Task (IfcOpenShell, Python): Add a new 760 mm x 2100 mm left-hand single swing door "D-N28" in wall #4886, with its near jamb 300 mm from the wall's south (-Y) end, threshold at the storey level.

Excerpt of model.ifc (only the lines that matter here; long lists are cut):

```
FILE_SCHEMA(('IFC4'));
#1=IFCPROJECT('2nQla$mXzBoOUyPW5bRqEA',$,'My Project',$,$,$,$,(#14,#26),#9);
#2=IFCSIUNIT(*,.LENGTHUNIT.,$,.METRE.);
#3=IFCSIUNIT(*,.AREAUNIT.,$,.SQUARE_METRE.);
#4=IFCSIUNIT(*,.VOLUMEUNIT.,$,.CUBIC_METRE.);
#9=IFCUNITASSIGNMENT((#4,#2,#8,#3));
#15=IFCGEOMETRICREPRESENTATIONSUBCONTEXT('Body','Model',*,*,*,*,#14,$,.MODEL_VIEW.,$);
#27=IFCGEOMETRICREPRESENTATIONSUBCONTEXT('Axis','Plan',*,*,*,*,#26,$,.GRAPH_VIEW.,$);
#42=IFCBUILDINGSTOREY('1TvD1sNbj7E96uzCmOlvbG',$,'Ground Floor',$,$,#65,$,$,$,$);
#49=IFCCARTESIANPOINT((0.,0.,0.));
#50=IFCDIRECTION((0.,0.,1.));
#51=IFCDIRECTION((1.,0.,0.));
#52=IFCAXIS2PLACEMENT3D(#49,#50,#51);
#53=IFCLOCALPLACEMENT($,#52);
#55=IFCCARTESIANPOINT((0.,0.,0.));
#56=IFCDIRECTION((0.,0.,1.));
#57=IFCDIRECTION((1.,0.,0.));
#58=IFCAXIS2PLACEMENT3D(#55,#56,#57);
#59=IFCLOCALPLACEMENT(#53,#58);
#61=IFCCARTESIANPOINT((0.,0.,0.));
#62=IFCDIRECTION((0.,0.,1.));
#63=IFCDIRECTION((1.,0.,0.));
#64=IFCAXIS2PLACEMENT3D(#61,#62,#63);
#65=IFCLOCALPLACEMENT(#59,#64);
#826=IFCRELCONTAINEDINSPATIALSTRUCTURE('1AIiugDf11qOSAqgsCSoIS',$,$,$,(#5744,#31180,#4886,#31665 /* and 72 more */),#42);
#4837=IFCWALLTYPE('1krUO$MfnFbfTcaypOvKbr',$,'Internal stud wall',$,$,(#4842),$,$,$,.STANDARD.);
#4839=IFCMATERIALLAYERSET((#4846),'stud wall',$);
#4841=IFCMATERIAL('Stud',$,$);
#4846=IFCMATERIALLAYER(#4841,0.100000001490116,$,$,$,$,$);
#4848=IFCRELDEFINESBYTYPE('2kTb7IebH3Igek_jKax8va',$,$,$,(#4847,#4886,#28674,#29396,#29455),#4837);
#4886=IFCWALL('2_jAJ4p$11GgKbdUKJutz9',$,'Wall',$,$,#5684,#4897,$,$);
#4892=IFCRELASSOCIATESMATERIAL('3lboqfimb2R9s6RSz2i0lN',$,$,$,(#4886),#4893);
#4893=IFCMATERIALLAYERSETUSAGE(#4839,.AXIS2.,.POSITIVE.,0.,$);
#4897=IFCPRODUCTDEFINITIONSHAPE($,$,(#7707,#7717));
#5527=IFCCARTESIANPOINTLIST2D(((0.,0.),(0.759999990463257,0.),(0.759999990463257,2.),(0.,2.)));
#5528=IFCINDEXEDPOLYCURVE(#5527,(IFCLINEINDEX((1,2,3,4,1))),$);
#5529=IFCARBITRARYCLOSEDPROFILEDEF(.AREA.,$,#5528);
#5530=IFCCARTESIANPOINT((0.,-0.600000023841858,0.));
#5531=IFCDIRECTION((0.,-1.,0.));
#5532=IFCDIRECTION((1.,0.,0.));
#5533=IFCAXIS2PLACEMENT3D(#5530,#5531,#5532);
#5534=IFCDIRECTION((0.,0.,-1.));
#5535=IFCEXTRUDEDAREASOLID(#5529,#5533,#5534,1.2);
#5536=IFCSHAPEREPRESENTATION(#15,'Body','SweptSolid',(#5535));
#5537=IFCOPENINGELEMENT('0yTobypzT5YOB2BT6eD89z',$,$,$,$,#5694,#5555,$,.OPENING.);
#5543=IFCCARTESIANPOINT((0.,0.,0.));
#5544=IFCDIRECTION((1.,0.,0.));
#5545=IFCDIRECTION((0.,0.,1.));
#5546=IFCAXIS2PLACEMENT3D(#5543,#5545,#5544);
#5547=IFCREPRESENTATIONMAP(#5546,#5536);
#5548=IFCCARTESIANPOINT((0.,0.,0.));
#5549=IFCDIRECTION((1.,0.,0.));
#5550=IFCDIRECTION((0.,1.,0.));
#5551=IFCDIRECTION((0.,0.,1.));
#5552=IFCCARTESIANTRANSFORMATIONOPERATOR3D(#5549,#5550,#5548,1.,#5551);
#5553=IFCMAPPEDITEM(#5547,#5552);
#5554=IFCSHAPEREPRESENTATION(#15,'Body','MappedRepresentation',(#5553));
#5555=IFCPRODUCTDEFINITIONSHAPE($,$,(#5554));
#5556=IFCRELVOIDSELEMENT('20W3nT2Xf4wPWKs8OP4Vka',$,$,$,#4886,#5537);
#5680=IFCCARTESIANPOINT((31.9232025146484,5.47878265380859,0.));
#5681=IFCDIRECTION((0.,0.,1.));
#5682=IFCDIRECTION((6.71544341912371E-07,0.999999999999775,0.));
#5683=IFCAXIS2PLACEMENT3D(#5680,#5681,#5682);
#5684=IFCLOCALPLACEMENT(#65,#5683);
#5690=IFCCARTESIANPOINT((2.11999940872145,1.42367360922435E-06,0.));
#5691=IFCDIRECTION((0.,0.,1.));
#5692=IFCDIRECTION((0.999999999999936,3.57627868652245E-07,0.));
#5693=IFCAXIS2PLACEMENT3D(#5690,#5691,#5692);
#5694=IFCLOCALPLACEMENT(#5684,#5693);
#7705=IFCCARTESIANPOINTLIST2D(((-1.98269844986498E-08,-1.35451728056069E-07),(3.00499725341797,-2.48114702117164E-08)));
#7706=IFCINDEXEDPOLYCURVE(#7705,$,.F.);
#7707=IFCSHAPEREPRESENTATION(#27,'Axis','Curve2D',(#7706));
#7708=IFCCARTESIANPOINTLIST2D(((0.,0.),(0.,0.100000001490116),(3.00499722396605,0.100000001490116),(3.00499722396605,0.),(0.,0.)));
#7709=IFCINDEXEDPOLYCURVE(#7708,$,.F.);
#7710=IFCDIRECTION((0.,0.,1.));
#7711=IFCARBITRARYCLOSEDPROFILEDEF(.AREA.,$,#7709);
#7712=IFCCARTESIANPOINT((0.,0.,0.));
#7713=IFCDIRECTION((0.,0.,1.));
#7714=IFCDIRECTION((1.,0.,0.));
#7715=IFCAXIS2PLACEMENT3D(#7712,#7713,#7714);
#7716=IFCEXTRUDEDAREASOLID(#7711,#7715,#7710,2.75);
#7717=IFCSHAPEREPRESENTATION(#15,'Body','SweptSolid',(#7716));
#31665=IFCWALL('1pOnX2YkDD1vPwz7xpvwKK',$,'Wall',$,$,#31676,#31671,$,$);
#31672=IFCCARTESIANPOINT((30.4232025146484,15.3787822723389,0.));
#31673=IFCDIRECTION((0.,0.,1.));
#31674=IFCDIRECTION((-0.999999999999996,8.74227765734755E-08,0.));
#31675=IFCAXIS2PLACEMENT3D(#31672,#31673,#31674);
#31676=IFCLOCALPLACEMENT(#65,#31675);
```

```python
import numpy as np
import ifcopenshell
import ifcopenshell.api.feature
import ifcopenshell.api.geometry
import ifcopenshell.api.root
import ifcopenshell.api.spatial
import ifcopenshell.geom
import ifcopenshell.util.element
import ifcopenshell.util.placement
import ifcopenshell.util.representation
import ifcopenshell.util.shape
import ifcopenshell.util.unit

model = ifcopenshell.open("model.ifc")
unit_scale = ifcopenshell.util.unit.calculate_unit_scale(model)
settings = ifcopenshell.geom.settings()


def volume(element):
    """Net volume in cubic metres, openings subtracted."""
    shape = ifcopenshell.geom.create_shape(settings, element)
    return ifcopenshell.util.shape.get_volume(shape.geometry)


wall = model.by_guid("2_jAJ4p$11GgKbdUKJutz9")
storey = ifcopenshell.util.element.get_container(wall, ifc_class="IfcBuildingStorey")
context = ifcopenshell.util.representation.get_context(model, "Model", "Body", "MODEL_VIEW")
before = volume(wall)

width, height, from_end, sill = 0.76, 2.1, 0.3, 0.0  # metres

# The wall runs along its own X axis, and the end named is its -X end.
wall_shape = ifcopenshell.geom.create_shape(settings, wall)
x, y, z = ifcopenshell.util.shape.get_vertices(wall_shape.geometry).T
start = x.min() + from_end
face, thickness = float(y.min()), float(y.max() - y.min())
wall_matrix = ifcopenshell.util.placement.get_local_placement(wall.ObjectPlacement)
level = ifcopenshell.util.placement.get_local_placement(storey.ObjectPlacement)[2, 3]


def in_wall(x, y):
    """Placement at x, y metres in the wall's axes, at sill height."""
    matrix = wall_matrix.copy()
    matrix[:, 3] = wall_matrix @ np.array([x / unit_scale, y / unit_scale, 0.0, 1.0])
    matrix[2, 3] = level + sill / unit_scale
    return matrix


# Opening: a box that overshoots both wall faces by 50 mm.
opening = ifcopenshell.api.root.create_entity(model, ifc_class="IfcOpeningElement", predefined_type="OPENING")
box = ifcopenshell.api.geometry.add_wall_representation(
    model, context=context, length=width, height=height, thickness=thickness + 0.1
)
ifcopenshell.api.geometry.assign_representation(model, product=opening, representation=box)
ifcopenshell.api.geometry.edit_object_placement(model, product=opening, matrix=in_wall(start, face - 0.05), is_si=False)
ifcopenshell.api.feature.add_feature(model, feature=opening, element=wall)

door = ifcopenshell.api.root.create_entity(model, ifc_class="IfcDoor", name="D-N28", predefined_type="DOOR")
door.OverallWidth, door.OverallHeight = width / unit_scale, height / unit_scale
door.OperationType = "SINGLE_SWING_LEFT"
body = ifcopenshell.api.geometry.add_door_representation(
    model,
    context=context,
    overall_width=door.OverallWidth,
    overall_height=door.OverallHeight,
    operation_type="SINGLE_SWING_LEFT",
    lining_properties={"LiningDepth": thickness / unit_scale, "ThresholdDepth": thickness / unit_scale},
)
ifcopenshell.api.geometry.assign_representation(model, product=door, representation=body)
ifcopenshell.api.spatial.assign_container(model, products=[door], relating_structure=storey)
ifcopenshell.api.feature.add_filling(model, opening=opening, element=door)

# The lining spans the wall, so the door starts at the wall face.
ifcopenshell.api.geometry.edit_object_placement(model, product=door, matrix=in_wall(start, face), is_si=False)

after = volume(wall)

print(f"wall volume {before:.3f} -> {after:.3f} m3")

model.write("model_rev.ifc")
```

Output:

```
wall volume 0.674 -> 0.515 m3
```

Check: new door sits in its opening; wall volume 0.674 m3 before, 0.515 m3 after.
